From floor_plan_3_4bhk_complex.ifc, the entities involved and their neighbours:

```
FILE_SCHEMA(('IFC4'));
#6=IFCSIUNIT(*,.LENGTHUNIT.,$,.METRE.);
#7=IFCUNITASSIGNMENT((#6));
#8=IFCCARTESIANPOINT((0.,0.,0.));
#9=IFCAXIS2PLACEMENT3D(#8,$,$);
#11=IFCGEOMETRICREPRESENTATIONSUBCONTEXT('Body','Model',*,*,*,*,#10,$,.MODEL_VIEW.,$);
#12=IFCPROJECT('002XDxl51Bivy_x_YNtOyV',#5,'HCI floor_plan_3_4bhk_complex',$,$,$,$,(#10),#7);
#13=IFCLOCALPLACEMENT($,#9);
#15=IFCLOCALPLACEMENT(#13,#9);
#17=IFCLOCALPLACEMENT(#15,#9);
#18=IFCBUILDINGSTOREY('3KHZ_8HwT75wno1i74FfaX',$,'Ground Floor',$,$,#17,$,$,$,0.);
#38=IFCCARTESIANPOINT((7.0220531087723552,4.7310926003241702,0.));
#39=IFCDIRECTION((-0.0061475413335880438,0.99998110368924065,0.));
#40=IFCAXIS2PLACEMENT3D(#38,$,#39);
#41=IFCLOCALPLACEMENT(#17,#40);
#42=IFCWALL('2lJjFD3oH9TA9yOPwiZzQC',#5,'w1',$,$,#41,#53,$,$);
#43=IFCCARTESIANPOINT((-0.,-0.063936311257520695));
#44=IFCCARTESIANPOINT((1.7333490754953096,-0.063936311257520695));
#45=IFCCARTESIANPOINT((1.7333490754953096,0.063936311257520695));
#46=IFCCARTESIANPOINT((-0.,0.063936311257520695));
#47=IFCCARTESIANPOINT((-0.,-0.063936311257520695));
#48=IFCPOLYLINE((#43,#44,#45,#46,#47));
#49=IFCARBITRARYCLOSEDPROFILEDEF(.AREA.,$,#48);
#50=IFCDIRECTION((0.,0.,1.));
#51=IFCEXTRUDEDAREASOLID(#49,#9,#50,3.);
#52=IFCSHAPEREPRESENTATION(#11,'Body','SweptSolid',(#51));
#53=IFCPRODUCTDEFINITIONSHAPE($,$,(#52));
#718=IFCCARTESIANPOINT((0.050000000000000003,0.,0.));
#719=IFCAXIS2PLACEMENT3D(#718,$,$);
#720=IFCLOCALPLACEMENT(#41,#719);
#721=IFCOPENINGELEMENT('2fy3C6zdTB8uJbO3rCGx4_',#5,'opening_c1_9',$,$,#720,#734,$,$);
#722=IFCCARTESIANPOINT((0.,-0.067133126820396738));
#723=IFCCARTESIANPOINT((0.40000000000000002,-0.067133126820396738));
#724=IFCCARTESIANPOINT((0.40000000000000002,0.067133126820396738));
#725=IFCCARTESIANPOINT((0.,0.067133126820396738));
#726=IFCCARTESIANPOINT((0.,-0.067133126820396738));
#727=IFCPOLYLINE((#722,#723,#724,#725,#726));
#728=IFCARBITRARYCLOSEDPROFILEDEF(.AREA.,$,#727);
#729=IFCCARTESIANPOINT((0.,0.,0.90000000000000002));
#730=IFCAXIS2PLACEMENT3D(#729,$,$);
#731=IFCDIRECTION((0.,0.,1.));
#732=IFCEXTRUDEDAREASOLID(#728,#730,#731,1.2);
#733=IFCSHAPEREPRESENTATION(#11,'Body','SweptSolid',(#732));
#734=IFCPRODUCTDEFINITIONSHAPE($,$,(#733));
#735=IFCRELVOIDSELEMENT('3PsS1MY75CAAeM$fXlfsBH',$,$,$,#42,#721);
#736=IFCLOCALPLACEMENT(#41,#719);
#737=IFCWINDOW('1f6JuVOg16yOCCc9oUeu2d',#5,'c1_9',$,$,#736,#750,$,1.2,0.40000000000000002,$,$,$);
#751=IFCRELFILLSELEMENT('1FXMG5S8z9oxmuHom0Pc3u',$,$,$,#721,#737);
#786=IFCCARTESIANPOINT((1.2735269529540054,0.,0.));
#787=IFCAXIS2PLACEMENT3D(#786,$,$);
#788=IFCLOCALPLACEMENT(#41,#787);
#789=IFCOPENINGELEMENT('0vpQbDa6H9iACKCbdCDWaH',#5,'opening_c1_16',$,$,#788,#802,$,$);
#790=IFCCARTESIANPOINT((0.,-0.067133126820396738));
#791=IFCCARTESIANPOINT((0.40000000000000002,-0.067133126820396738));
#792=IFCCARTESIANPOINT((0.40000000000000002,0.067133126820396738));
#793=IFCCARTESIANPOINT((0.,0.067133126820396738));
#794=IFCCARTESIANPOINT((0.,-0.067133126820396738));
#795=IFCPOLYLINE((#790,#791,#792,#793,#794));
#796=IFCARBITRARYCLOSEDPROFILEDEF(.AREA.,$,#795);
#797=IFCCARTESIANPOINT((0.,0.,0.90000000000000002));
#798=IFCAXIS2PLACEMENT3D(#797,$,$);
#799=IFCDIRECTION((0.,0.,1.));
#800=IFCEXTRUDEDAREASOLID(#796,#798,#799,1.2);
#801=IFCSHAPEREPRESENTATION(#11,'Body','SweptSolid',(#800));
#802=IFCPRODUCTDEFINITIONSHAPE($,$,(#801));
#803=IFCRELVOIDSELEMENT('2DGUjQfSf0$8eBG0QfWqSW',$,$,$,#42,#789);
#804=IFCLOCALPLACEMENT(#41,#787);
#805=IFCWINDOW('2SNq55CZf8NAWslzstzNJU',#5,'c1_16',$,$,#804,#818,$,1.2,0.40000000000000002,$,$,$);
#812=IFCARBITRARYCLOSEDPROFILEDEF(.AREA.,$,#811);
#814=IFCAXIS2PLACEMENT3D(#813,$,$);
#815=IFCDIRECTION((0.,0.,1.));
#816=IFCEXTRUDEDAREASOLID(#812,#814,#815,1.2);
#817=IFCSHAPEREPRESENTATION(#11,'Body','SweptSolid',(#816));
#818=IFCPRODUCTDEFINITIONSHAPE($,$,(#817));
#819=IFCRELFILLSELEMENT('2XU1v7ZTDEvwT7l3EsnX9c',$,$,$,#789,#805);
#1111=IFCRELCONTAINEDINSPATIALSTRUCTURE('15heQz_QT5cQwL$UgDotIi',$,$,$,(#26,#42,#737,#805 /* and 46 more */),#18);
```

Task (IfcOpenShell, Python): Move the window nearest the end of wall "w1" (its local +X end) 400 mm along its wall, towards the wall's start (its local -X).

```python
import ifcopenshell
import ifcopenshell.api.geometry
import ifcopenshell.util.placement

model = ifcopenshell.open("floor_plan_3_4bhk_complex.ifc")

window = model.by_guid("2SNq55CZf8NAWslzstzNJU")
opening = window.FillsVoids[0].RelatingOpeningElement
wall = opening.VoidsElements[0].RelatingBuildingElement

wall_matrix = ifcopenshell.util.placement.get_local_placement(wall.ObjectPlacement)
shift = wall_matrix[:3, 0] * -0.4
before = ifcopenshell.util.placement.get_local_placement(window.ObjectPlacement)[:3, 3].copy()

# The window is not placed relative to its opening, so move both.
for product in (opening, window):
    matrix = ifcopenshell.util.placement.get_local_placement(product.ObjectPlacement)
    matrix[:3, 3] += shift
    ifcopenshell.api.geometry.edit_object_placement(model, product=product, matrix=matrix, is_si=False)

after = ifcopenshell.util.placement.get_local_placement(window.ObjectPlacement)[:3, 3]
print("window moved by", (after - before).round(3) + 0.0)

model.write("floor_plan_3_4bhk_complex_rev.ifc")
```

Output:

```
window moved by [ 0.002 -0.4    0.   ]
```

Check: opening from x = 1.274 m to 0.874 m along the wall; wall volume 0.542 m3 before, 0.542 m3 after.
